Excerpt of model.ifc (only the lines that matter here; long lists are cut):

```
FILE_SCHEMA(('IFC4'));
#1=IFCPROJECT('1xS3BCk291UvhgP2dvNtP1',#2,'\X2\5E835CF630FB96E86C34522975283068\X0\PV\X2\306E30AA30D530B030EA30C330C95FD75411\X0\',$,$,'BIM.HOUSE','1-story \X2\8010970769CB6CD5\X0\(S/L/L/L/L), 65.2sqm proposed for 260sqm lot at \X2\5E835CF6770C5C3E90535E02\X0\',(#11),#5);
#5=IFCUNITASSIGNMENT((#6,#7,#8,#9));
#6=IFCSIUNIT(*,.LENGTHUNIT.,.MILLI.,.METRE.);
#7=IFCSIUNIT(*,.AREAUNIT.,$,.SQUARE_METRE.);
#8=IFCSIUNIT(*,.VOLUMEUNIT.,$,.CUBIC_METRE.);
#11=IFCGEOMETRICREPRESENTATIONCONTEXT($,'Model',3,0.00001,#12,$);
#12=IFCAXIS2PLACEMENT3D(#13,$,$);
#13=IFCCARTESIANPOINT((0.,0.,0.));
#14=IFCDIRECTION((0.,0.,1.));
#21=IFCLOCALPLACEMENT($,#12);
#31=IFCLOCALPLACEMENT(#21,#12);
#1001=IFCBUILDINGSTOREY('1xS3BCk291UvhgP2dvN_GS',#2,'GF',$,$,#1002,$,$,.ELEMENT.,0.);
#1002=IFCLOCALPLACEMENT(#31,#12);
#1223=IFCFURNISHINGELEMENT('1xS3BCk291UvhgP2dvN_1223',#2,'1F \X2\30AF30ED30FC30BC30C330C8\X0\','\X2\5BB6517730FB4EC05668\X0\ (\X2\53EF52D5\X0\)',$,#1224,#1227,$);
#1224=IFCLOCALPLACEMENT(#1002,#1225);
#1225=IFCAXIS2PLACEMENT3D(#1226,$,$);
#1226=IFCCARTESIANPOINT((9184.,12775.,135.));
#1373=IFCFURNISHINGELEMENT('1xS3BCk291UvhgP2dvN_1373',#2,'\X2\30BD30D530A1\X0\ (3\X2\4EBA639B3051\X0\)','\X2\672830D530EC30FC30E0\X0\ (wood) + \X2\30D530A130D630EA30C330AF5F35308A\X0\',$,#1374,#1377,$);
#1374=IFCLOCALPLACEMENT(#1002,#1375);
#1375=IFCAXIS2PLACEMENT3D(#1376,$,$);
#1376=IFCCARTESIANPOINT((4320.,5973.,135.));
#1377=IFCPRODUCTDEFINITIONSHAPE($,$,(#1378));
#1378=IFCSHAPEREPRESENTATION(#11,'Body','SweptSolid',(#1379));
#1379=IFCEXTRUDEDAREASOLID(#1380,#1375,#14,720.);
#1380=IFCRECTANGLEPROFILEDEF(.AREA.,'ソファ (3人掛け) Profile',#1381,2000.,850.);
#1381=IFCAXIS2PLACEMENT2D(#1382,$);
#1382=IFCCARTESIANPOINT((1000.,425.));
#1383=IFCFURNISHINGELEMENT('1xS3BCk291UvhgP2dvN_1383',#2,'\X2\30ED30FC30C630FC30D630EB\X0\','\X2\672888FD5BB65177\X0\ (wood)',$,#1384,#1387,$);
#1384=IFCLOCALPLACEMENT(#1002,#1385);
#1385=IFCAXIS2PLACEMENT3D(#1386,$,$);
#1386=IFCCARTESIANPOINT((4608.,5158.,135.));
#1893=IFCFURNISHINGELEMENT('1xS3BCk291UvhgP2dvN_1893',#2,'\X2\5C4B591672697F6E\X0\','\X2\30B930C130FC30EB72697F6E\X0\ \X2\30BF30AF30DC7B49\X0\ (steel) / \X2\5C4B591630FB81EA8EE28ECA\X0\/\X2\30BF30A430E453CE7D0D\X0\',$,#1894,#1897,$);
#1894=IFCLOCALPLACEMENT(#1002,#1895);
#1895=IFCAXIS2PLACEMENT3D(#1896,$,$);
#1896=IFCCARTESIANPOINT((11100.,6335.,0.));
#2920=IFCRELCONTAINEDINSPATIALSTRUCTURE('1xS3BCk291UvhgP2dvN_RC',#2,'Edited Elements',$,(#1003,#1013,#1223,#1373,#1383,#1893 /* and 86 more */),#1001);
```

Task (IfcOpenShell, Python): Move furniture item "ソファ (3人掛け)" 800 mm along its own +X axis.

```python
import ifcopenshell
import ifcopenshell.api.geometry
import ifcopenshell.util.placement

model = ifcopenshell.open("model.ifc")

item = model.by_guid("1xS3BCk291UvhgP2dvN_1373")
matrix = ifcopenshell.util.placement.get_local_placement(item.ObjectPlacement)
matrix[:3, 3] += matrix[:3, 0] * 800.0
ifcopenshell.api.geometry.edit_object_placement(model, product=item, matrix=matrix, is_si=False)

print(ifcopenshell.util.placement.get_local_placement(item.ObjectPlacement).round(3) + 0.0)

model.write("model_v2.ifc")
```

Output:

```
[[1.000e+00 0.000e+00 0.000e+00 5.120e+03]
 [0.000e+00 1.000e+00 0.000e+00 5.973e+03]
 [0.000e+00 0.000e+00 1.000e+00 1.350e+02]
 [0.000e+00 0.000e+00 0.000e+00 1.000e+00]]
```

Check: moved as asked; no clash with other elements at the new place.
